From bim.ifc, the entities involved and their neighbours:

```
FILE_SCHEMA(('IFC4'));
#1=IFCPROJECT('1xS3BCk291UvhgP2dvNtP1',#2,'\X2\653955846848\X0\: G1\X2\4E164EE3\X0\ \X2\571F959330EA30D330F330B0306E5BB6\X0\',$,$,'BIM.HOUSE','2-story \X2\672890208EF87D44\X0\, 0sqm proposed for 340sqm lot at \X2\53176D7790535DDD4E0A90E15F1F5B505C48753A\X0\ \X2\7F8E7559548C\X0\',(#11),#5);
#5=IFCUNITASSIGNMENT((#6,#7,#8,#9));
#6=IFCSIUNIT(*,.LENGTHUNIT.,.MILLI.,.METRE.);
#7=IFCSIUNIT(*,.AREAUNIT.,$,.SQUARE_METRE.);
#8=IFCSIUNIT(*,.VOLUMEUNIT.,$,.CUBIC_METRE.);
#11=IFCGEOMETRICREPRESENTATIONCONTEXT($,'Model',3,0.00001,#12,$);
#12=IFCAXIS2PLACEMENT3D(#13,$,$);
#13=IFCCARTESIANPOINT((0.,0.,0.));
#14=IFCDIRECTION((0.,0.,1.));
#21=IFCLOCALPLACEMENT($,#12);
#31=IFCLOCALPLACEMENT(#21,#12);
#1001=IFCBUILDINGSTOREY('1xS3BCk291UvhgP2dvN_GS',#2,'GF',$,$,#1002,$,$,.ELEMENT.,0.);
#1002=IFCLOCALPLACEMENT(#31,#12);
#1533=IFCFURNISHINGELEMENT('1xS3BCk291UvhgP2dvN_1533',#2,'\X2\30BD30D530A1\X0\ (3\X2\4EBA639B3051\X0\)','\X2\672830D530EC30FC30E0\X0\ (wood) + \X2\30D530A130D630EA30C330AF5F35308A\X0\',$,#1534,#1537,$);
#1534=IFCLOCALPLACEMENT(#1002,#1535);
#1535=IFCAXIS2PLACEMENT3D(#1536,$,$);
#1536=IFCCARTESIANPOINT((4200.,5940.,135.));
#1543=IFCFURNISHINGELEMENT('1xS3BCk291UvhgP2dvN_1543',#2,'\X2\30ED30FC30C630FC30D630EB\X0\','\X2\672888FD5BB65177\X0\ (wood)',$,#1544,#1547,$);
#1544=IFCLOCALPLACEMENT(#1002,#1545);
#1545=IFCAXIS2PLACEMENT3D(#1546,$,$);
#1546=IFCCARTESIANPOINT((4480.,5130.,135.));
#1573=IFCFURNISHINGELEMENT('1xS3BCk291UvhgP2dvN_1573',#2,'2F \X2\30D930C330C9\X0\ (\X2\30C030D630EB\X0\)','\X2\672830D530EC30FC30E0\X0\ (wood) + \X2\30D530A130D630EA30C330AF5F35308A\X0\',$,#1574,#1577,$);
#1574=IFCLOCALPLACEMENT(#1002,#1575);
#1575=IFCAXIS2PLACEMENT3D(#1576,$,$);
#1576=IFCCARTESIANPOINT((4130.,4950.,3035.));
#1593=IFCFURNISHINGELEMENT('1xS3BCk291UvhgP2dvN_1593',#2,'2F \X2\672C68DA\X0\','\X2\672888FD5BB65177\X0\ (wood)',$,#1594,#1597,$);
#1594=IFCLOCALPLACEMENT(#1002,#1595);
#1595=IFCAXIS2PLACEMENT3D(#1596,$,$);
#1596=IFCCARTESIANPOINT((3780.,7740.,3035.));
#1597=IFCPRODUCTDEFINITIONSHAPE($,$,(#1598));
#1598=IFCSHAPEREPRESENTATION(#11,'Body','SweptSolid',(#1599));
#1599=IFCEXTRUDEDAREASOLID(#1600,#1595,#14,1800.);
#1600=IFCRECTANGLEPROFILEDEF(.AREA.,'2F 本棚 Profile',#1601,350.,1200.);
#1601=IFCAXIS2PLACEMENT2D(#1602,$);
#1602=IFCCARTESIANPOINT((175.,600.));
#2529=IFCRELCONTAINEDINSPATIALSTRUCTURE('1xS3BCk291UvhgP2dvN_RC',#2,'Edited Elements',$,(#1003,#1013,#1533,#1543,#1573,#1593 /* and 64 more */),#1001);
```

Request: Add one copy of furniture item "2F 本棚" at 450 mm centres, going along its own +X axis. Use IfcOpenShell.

```python
import ifcopenshell
import ifcopenshell.api.geometry
import ifcopenshell.api.root
import ifcopenshell.util.element
import ifcopenshell.util.placement
import ifcopenshell.util.unit

model = ifcopenshell.open("bim.ifc")
unit_scale = ifcopenshell.util.unit.calculate_unit_scale(model)


def reuse_history(source, copy):
    """copy_class also copies each property set's owner history, people and application; keep the originals."""
    for rel in copy.IsDefinedBy:
        if rel.is_a("IfcRelDefinesByProperties") and (history := rel.RelatingPropertyDefinition.OwnerHistory):
            rel.RelatingPropertyDefinition.OwnerHistory = source.OwnerHistory
            ifcopenshell.util.element.remove_deep2(model, history)


source = model.by_guid("1xS3BCk291UvhgP2dvN_1593")
base = ifcopenshell.util.placement.get_local_placement(source.ObjectPlacement)
step = base[:3, 0] * 0.45 / unit_scale

for i in range(1, 2):
    copy = ifcopenshell.api.root.copy_class(model, product=source)
    copy.Representation = ifcopenshell.util.element.copy_deep(
        model, source.Representation, exclude=["IfcGeometricRepresentationContext", "IfcRepresentationMap"]
    )
    reuse_history(source, copy)
    matrix = base.copy()
    matrix[:3, 3] += i * step
    print("added at", matrix[:3, 3].round(3) + 0.0)
    ifcopenshell.api.geometry.edit_object_placement(model, product=copy, matrix=matrix, is_si=False)

model.write("bim_updated.ifc")
```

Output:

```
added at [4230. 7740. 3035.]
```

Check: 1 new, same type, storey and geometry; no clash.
